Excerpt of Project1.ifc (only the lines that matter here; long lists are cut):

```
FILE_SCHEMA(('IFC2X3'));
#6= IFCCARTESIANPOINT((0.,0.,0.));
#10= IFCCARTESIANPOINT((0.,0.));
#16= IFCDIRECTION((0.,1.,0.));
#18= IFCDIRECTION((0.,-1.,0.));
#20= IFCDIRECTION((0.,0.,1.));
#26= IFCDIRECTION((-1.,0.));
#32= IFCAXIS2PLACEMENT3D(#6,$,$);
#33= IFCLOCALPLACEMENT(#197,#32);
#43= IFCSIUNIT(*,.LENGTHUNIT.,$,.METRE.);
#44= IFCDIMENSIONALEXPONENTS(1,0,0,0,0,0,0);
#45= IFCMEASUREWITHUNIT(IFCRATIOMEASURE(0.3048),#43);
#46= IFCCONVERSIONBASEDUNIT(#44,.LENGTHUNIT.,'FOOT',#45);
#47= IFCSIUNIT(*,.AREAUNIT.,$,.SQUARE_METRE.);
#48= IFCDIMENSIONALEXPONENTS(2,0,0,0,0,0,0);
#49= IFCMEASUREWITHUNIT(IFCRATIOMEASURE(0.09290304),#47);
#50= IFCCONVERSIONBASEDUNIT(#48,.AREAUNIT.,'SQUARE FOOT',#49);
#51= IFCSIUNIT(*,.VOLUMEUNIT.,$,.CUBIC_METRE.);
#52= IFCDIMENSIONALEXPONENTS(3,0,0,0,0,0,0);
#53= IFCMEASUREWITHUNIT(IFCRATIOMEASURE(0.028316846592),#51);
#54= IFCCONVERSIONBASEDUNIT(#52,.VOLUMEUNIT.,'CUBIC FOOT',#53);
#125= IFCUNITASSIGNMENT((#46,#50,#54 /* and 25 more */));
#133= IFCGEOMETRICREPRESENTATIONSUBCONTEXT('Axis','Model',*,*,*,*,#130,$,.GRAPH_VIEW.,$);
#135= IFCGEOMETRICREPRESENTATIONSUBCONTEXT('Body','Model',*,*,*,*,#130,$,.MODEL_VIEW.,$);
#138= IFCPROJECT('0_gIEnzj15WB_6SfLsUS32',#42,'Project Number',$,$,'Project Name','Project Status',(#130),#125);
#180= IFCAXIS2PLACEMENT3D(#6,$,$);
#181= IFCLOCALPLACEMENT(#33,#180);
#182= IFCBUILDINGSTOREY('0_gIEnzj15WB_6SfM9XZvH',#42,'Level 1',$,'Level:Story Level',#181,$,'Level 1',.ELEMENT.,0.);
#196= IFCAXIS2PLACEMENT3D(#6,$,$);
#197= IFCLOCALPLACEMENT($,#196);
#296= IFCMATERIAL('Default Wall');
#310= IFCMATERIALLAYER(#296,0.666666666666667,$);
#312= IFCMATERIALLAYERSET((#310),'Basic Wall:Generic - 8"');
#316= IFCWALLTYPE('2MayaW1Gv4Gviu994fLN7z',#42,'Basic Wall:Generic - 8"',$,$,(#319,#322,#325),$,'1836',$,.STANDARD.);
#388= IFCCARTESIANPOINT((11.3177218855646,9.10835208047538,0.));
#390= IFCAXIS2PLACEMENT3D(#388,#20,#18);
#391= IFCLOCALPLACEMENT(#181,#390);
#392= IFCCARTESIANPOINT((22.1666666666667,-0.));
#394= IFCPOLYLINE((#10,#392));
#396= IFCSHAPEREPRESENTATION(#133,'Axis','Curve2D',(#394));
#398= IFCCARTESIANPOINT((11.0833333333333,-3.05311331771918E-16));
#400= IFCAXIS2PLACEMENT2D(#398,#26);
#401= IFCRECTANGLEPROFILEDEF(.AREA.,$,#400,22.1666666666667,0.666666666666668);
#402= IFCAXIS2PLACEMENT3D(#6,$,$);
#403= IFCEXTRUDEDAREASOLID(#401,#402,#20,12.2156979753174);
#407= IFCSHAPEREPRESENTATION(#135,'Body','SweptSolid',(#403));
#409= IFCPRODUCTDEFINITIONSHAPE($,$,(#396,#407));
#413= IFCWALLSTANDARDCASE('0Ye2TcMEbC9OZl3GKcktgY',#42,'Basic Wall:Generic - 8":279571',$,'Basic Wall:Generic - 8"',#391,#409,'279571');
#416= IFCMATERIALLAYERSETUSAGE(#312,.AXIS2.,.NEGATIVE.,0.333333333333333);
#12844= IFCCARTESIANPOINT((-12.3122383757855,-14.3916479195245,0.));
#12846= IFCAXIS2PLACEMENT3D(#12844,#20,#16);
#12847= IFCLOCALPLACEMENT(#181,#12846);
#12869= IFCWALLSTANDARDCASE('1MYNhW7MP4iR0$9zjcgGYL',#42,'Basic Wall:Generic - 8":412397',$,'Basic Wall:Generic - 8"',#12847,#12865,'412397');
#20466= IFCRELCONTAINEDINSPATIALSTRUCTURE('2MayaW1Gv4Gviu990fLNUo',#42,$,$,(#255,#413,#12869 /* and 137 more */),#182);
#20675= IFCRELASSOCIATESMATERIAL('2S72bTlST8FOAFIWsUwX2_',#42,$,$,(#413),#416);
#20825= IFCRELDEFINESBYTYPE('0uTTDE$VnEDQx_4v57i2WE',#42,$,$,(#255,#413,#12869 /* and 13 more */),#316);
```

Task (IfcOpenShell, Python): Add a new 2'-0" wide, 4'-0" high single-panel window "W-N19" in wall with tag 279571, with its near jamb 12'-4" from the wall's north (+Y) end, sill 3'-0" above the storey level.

```python
import numpy as np
import ifcopenshell
import ifcopenshell.api.feature
import ifcopenshell.api.geometry
import ifcopenshell.api.root
import ifcopenshell.api.spatial
import ifcopenshell.api.type
import ifcopenshell.geom
import ifcopenshell.util.element
import ifcopenshell.util.placement
import ifcopenshell.util.representation
import ifcopenshell.util.shape
import ifcopenshell.util.unit

model = ifcopenshell.open("Project1.ifc")
unit_scale = ifcopenshell.util.unit.calculate_unit_scale(model)
settings = ifcopenshell.geom.settings()


def volume(element):
    """Net volume in cubic metres, openings subtracted."""
    shape = ifcopenshell.geom.create_shape(settings, element)
    return ifcopenshell.util.shape.get_volume(shape.geometry)


wall = model.by_id(413)
storey = ifcopenshell.util.element.get_container(wall, ifc_class="IfcBuildingStorey")
context = ifcopenshell.util.representation.get_context(model, "Model", "Body", "MODEL_VIEW")
before = volume(wall)

width, height, from_end, sill = 0.6096, 1.2192, 3.7592, 0.9144  # metres

# The wall runs along its own X axis, and the end named is its -X end.
wall_shape = ifcopenshell.geom.create_shape(settings, wall)
x, y, z = ifcopenshell.util.shape.get_vertices(wall_shape.geometry).T
start = x.min() + from_end
face, thickness = float(y.min()), float(y.max() - y.min())
wall_matrix = ifcopenshell.util.placement.get_local_placement(wall.ObjectPlacement)
level = ifcopenshell.util.placement.get_local_placement(storey.ObjectPlacement)[2, 3]


def in_wall(x, y):
    """Placement at x, y metres in the wall's axes, at sill height."""
    matrix = wall_matrix.copy()
    matrix[:, 3] = wall_matrix @ np.array([x / unit_scale, y / unit_scale, 0.0, 1.0])
    matrix[2, 3] = level + sill / unit_scale
    return matrix


# Opening: a box that overshoots both wall faces by 50 mm.
opening = ifcopenshell.api.root.create_entity(model, ifc_class="IfcOpeningElement")
box = ifcopenshell.api.geometry.add_wall_representation(
    model, context=context, length=width, height=height, thickness=thickness + 0.1
)
ifcopenshell.api.geometry.assign_representation(model, product=opening, representation=box)
ifcopenshell.api.geometry.edit_object_placement(model, product=opening, matrix=in_wall(start, face - 0.05), is_si=False)
ifcopenshell.api.feature.add_feature(model, feature=opening, element=wall)

window = ifcopenshell.api.root.create_entity(model, ifc_class="IfcWindow", name="W-N19")
window.OverallWidth, window.OverallHeight = width / unit_scale, height / unit_scale
body = ifcopenshell.api.geometry.add_window_representation(
    model,
    context=context,
    overall_width=window.OverallWidth,
    overall_height=window.OverallHeight,
    partition_type="SINGLE_PANEL",
)
ifcopenshell.api.geometry.assign_representation(model, product=window, representation=body)
ifcopenshell.api.spatial.assign_container(model, products=[window], relating_structure=storey)
fills = ifcopenshell.api.feature.add_filling(model, opening=opening, element=window)
fills.OwnerHistory = window.OwnerHistory  # required in IFC2X3

# IFC2X3 keeps the operation on the window style.
style = ifcopenshell.api.root.create_entity(model, ifc_class="IfcWindowStyle", name="W-N19")
style.OperationType, style.ConstructionType = "SINGLE_PANEL", "NOTDEFINED"
style.ParameterTakesPrecedence = style.Sizeable = False
ifcopenshell.api.type.assign_type(model, related_objects=[window], relating_type=style)

# Centre the window in the wall's thickness.
ifcopenshell.api.geometry.edit_object_placement(model, product=window, matrix=in_wall(start, face), is_si=False)
window_shape = ifcopenshell.geom.create_shape(settings, window)
depth = ifcopenshell.util.shape.get_vertices(window_shape.geometry)[:, 1]
offset = face + thickness / 2 - (depth.min() + depth.max()) / 2
ifcopenshell.api.geometry.edit_object_placement(model, product=window, matrix=in_wall(start, offset), is_si=False)

after = volume(wall)

print(f"wall volume {before:.3f} -> {after:.3f} m3")

model.write("Project1_rev.ifc")
```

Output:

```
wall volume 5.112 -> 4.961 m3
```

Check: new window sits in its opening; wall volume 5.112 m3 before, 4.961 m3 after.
